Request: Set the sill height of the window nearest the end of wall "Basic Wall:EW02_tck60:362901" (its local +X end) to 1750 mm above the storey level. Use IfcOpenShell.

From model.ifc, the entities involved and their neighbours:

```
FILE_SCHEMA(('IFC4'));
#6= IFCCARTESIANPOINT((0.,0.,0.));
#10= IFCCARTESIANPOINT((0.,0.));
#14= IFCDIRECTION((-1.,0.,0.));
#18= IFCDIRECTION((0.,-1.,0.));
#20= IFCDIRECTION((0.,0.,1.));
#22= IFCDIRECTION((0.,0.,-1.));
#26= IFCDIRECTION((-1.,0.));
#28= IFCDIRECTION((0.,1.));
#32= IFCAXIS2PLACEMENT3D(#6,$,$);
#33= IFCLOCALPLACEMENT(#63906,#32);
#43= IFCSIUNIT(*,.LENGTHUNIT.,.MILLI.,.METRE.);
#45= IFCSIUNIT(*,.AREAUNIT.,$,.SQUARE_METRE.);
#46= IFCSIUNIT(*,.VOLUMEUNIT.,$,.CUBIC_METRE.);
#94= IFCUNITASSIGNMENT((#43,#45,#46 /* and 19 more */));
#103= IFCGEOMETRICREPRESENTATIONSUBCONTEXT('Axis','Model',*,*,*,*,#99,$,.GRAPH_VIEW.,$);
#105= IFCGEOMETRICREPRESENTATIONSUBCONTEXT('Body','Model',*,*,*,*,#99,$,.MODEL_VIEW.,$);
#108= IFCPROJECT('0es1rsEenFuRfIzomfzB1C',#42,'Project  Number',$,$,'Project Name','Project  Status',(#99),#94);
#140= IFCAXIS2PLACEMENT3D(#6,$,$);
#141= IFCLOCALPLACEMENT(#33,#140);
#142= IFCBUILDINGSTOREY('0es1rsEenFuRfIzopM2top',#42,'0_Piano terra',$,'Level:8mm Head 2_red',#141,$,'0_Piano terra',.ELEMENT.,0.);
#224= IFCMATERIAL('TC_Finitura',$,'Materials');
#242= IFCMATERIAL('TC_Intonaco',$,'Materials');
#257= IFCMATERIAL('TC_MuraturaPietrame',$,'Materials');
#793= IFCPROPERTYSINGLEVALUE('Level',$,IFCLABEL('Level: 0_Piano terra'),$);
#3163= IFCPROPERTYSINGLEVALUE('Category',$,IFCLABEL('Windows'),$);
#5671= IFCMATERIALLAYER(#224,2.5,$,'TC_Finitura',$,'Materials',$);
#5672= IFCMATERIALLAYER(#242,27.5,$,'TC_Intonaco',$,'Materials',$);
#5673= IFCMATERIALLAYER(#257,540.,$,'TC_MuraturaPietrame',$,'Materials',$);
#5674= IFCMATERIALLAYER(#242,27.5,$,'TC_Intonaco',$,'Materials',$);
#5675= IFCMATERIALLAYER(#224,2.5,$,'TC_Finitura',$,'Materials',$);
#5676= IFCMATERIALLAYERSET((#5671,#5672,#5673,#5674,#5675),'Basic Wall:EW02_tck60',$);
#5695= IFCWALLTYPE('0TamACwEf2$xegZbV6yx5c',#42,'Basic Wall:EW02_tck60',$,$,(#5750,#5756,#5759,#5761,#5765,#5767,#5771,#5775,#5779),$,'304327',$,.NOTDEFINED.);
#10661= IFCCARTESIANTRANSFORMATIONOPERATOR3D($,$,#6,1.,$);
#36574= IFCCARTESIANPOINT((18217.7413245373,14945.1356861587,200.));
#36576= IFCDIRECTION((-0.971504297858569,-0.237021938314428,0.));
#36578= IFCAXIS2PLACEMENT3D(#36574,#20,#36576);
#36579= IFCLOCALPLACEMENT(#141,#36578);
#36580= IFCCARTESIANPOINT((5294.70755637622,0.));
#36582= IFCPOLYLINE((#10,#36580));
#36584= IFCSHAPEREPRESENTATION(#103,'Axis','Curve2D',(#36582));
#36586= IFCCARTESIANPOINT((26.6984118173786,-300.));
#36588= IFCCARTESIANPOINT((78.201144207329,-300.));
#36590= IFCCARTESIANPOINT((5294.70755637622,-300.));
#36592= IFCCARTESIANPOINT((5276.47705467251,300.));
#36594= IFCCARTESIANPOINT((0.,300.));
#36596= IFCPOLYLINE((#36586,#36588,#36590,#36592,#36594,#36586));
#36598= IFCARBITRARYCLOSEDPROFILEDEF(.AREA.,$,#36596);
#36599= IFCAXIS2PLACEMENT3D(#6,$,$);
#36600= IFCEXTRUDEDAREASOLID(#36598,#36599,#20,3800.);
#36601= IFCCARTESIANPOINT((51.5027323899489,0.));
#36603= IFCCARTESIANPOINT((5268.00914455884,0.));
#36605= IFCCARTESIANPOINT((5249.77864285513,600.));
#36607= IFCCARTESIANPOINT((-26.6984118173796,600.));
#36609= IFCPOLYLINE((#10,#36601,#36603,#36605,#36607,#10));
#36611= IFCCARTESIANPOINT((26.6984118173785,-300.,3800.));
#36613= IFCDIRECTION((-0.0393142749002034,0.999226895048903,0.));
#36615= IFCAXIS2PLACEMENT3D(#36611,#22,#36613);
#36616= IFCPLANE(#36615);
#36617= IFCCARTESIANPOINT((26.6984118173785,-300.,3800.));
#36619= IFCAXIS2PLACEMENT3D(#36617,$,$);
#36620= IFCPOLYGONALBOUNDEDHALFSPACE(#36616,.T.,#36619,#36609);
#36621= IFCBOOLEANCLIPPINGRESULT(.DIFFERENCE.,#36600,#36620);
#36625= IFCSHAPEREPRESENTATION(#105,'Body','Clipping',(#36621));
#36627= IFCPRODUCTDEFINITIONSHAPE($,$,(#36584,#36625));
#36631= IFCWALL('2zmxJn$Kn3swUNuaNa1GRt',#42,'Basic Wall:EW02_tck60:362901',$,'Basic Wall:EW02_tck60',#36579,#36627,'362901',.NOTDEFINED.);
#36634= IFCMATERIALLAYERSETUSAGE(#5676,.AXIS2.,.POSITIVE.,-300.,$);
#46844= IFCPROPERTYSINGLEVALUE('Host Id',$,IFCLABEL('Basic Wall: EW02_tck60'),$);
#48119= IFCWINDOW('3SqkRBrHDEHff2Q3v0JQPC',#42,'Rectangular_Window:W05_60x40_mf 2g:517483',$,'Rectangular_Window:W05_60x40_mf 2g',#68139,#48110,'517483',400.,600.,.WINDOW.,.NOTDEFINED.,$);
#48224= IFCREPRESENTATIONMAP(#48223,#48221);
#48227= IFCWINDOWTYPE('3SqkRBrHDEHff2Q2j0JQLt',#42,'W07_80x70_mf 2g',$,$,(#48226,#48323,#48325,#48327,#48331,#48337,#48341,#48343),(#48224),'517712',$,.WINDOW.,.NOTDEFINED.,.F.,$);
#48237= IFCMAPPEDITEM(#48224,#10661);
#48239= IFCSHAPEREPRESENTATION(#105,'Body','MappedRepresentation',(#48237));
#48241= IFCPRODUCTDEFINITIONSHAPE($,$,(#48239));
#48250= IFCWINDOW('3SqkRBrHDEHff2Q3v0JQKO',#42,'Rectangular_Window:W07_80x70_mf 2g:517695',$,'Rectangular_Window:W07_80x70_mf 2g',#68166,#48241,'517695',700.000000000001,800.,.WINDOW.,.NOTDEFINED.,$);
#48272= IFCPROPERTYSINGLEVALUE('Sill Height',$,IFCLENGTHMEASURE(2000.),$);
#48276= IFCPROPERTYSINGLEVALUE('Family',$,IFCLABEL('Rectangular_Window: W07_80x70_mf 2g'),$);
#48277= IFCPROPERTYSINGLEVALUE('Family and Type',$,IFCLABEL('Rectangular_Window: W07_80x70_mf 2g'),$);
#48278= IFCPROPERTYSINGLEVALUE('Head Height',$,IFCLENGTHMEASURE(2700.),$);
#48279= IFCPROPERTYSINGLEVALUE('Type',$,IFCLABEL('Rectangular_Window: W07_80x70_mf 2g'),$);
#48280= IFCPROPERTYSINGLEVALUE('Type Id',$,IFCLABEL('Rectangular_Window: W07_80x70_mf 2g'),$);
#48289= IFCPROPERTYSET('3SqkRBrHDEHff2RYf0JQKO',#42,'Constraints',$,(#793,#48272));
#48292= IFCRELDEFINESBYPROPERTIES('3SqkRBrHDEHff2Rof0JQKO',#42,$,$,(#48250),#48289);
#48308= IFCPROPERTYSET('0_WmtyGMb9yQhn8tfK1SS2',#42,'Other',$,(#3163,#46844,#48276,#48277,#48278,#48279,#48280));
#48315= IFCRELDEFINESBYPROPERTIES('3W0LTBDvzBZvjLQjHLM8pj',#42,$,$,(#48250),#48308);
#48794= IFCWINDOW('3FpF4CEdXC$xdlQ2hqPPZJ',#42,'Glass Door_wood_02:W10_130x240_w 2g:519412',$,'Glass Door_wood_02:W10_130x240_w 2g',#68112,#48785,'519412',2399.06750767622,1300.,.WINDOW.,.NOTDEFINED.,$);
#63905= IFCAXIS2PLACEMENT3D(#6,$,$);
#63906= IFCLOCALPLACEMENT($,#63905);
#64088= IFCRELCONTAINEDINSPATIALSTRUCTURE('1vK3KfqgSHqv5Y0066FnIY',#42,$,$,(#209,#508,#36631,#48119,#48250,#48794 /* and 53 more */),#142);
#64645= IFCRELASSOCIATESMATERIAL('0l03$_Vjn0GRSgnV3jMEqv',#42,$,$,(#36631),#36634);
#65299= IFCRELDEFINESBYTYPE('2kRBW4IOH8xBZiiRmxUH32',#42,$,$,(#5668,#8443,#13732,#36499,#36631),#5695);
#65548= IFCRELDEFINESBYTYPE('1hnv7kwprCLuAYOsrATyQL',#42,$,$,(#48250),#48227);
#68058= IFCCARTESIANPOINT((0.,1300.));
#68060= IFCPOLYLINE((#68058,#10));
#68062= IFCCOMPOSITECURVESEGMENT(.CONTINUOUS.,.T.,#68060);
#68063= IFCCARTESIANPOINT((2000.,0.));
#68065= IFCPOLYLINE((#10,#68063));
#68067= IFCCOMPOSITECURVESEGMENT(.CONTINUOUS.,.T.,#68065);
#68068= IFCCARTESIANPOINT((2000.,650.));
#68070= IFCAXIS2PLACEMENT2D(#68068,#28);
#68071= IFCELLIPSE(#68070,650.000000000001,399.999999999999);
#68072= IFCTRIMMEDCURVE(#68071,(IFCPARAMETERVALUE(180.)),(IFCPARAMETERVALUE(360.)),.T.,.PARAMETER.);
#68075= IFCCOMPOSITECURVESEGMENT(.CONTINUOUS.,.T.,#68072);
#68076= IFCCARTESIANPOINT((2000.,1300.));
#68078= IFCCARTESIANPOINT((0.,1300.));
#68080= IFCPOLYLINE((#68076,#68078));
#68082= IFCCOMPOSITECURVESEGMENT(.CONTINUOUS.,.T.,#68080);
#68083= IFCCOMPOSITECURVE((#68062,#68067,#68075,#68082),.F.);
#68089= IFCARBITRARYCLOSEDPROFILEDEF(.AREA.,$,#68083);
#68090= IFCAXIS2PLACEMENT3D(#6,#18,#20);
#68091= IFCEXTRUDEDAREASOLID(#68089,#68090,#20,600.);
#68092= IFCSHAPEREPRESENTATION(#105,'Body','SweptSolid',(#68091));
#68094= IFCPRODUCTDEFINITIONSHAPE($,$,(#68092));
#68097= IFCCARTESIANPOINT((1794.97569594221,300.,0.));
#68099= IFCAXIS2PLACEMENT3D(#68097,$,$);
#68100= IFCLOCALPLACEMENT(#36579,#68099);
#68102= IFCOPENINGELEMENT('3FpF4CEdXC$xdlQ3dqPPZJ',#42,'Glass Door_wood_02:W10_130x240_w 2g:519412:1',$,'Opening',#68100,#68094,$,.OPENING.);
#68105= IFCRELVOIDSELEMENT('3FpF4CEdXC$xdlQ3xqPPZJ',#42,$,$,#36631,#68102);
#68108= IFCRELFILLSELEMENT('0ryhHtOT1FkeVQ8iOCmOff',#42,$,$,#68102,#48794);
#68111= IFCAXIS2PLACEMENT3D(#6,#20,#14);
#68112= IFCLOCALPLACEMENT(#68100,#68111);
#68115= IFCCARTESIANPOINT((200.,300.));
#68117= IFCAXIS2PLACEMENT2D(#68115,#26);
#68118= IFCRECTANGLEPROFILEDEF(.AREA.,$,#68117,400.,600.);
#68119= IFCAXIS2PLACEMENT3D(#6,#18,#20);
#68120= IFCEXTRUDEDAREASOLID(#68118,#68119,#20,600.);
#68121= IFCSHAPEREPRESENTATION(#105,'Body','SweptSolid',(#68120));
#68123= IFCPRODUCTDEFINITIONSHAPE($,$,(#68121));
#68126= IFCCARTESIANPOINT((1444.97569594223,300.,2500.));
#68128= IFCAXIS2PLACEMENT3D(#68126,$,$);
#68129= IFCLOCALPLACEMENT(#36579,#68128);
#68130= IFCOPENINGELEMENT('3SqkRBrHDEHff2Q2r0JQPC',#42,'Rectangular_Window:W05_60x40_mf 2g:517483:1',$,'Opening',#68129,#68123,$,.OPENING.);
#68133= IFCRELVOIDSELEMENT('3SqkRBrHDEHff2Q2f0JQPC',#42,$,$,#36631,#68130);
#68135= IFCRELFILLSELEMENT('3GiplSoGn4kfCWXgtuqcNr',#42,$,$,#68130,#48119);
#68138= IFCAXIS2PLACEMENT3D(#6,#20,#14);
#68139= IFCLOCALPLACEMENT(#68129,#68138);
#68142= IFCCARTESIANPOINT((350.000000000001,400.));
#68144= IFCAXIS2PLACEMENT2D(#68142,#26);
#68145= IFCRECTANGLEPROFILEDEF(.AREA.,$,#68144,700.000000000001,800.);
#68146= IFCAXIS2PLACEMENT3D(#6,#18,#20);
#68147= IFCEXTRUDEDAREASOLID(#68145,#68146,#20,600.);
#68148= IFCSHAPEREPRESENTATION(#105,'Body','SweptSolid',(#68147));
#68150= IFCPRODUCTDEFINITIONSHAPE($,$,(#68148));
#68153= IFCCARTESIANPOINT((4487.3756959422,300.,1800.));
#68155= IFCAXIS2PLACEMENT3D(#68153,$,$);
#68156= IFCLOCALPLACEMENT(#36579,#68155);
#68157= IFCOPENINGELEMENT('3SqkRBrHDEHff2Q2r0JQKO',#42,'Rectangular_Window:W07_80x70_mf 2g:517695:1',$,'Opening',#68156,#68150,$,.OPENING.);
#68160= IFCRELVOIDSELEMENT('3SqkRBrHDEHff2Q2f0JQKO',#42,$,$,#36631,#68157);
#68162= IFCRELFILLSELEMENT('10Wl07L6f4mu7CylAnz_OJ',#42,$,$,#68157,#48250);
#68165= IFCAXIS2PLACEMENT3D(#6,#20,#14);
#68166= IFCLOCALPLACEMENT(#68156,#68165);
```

```python
import numpy as np
import ifcopenshell
import ifcopenshell.api.geometry
import ifcopenshell.api.pset
import ifcopenshell.geom
import ifcopenshell.util.element
import ifcopenshell.util.placement
import ifcopenshell.util.shape
import ifcopenshell.util.unit

model = ifcopenshell.open("model.ifc")
unit_scale = ifcopenshell.util.unit.calculate_unit_scale(model)

window = model.by_guid("3SqkRBrHDEHff2Q3v0JQKO")
opening = window.FillsVoids[0].RelatingOpeningElement
storey = ifcopenshell.util.element.get_container(window, ifc_class="IfcBuildingStorey")
level = ifcopenshell.util.placement.get_local_placement(storey.ObjectPlacement)[2, 3]

# The opening's origin need not be at the sill, so measure its lowest point.
shape = ifcopenshell.geom.create_shape(ifcopenshell.geom.settings(), opening)
bottom = ifcopenshell.util.shape.get_shape_bottom_elevation(shape, shape.geometry) / unit_scale
dz = level + 1.75 / unit_scale - bottom

shift = np.array([0.0, 0.0, dz])
# The window is placed relative to its opening, so it follows when the opening moves.
matrix = ifcopenshell.util.placement.get_local_placement(opening.ObjectPlacement)
matrix[:3, 3] += shift
ifcopenshell.api.geometry.edit_object_placement(
    model, product=opening, matrix=matrix, is_si=False, should_transform_children=True
)

# Keep the stored heights in step.
pset = model.by_id(ifcopenshell.util.element.get_pset(window, "Constraints", should_inherit=False)["id"])
ifcopenshell.api.pset.edit_pset(model, pset=pset, properties={
    "Sill Height": model.create_entity("IfcLengthMeasure", ifcopenshell.util.element.get_pset(window, "Constraints", "Sill Height") + dz),
})
pset = model.by_id(ifcopenshell.util.element.get_pset(window, "Other", should_inherit=False)["id"])
ifcopenshell.api.pset.edit_pset(model, pset=pset, properties={
    "Head Height": model.create_entity("IfcLengthMeasure", ifcopenshell.util.element.get_pset(window, "Other", "Head Height") + dz),
})

print(f"moved by {dz * unit_scale:+.3f} m")

model.write("model_v2.ifc")
```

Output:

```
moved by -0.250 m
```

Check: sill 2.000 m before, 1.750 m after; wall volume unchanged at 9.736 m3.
